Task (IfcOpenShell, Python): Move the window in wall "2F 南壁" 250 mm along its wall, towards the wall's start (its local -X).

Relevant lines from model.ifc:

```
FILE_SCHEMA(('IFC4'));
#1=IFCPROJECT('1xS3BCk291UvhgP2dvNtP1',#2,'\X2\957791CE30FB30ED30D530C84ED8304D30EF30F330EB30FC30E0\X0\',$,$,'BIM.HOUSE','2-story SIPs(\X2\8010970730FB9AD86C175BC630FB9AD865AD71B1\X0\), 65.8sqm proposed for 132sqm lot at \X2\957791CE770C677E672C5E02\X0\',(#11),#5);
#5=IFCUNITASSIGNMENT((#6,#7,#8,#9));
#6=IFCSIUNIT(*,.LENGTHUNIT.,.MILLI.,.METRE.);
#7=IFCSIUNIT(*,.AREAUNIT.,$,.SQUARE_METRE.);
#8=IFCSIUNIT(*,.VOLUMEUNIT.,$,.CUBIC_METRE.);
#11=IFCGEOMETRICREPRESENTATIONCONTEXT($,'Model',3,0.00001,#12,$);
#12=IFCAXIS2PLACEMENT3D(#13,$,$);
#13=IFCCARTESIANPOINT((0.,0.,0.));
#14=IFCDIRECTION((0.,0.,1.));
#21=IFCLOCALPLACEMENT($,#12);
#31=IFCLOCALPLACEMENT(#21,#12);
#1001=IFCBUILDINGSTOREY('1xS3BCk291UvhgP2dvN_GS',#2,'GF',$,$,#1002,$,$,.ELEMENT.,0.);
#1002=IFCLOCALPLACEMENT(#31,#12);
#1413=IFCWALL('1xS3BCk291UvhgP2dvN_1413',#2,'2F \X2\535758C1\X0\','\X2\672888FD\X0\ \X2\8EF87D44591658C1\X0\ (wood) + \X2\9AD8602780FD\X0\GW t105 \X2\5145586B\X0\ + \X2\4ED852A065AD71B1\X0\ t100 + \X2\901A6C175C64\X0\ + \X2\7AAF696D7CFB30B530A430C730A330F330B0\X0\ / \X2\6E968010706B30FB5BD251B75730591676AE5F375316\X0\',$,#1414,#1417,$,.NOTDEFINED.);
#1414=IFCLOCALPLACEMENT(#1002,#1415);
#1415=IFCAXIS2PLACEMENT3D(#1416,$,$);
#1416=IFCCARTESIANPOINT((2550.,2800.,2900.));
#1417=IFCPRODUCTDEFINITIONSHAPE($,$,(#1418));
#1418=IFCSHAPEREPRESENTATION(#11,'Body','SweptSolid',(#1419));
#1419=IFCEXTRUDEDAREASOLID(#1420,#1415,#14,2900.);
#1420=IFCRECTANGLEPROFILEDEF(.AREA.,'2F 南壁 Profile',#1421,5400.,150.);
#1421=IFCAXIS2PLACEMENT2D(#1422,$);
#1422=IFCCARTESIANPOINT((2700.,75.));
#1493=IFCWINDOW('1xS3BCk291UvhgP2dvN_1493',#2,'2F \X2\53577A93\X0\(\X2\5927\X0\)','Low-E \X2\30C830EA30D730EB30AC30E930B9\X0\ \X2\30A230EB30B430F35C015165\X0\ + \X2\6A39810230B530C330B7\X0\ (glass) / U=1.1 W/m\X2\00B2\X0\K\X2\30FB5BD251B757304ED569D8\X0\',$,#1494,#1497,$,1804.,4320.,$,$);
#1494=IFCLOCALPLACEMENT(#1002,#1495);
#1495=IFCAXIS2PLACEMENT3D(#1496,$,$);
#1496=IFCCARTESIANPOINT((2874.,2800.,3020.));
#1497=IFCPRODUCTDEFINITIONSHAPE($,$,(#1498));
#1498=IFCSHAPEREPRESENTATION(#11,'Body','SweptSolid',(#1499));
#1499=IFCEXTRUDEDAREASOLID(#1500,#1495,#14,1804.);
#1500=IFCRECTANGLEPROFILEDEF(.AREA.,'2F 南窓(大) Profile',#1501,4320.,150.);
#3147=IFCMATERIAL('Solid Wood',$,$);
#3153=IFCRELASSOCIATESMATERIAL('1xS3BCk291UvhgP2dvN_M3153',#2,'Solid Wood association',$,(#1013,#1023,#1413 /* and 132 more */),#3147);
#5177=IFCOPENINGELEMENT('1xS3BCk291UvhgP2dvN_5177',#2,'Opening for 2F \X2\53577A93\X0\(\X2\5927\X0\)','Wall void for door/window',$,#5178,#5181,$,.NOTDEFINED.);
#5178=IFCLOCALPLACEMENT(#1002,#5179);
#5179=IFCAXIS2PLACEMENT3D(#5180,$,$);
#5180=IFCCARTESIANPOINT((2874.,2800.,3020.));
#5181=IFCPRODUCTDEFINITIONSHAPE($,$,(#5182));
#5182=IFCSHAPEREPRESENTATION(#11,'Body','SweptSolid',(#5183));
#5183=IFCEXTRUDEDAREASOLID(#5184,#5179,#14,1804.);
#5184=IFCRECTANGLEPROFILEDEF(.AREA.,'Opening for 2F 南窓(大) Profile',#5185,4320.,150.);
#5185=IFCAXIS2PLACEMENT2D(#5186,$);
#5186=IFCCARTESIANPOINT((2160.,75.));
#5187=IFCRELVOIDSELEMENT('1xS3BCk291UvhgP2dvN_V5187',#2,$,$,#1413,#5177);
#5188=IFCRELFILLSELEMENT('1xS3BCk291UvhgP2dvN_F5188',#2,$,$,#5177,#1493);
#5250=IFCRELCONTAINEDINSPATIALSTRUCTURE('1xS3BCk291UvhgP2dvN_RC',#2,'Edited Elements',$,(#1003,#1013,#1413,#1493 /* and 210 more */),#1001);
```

```python
import ifcopenshell
import ifcopenshell.api.geometry
import ifcopenshell.util.placement
import ifcopenshell.util.unit

model = ifcopenshell.open("model.ifc")
unit_scale = ifcopenshell.util.unit.calculate_unit_scale(model)

window = model.by_guid("1xS3BCk291UvhgP2dvN_1493")
opening = window.FillsVoids[0].RelatingOpeningElement
wall = opening.VoidsElements[0].RelatingBuildingElement

wall_matrix = ifcopenshell.util.placement.get_local_placement(wall.ObjectPlacement)
shift = wall_matrix[:3, 0] * -0.25 / unit_scale
before = ifcopenshell.util.placement.get_local_placement(window.ObjectPlacement)[:3, 3].copy()

# The window is not placed relative to its opening, so move both.
for product in (opening, window):
    matrix = ifcopenshell.util.placement.get_local_placement(product.ObjectPlacement)
    matrix[:3, 3] += shift
    ifcopenshell.api.geometry.edit_object_placement(model, product=product, matrix=matrix, is_si=False)

after = ifcopenshell.util.placement.get_local_placement(window.ObjectPlacement)[:3, 3]
print("window moved by", (after - before).round(3) + 0.0)

model.write("model_edited.ifc")
```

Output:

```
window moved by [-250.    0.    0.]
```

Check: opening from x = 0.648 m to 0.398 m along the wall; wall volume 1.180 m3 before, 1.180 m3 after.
